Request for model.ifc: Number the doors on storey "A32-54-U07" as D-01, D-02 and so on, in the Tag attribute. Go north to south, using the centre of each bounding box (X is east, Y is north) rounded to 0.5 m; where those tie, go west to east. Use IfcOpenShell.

First a look at what the model holds.

```python
import ifcopenshell
import ifcopenshell.util.element
import ifcopenshell.util.placement

model = ifcopenshell.open("model.ifc")
print(model.schema)
storey = next(s for s in model.by_type("IfcBuildingStorey") if s.Name == "A32-54-U07")
doors = [e for e in ifcopenshell.util.element.get_decomposition(storey) if e.is_a("IfcDoor")]
for e in sorted(doors, key=lambda e: e.id()):
    origin = ifcopenshell.util.placement.get_local_placement(e.ObjectPlacement)[:3, 3]
    print(e.id(), e.Tag, e.Name, origin.round(2) + 0.0, sep=" | ")
```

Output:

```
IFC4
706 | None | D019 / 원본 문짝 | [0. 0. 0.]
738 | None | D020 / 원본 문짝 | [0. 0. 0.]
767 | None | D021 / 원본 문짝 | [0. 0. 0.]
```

```python
import ifcopenshell
import ifcopenshell.geom
import ifcopenshell.util.element
import ifcopenshell.util.shape

model = ifcopenshell.open("model.ifc")
settings = ifcopenshell.geom.settings()
settings.set("use-world-coords", True)


def centre(element):
    shape = ifcopenshell.geom.create_shape(settings, element)
    return ifcopenshell.util.shape.get_bbox_centroid(shape.geometry)


storey = next(s for s in model.by_type("IfcBuildingStorey") if s.Name == "A32-54-U07")
doors = [e for e in ifcopenshell.util.element.get_decomposition(storey) if e.is_a("IfcDoor")]

# Insertion points can sit at a corner or the storey origin, so sort by the geometry (in metres).
centres = {e: centre(e) for e in doors}
doors.sort(key=lambda e: (-round(centres[e][1] / 0.5), centres[e][0]))

for i, e in enumerate(doors, start=1):
    number = f"D-{i:02d}"
    e.Tag = number
    print(e.id(), number)

model.write("model_edited.ifc")
```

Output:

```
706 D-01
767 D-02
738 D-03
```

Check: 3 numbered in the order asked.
